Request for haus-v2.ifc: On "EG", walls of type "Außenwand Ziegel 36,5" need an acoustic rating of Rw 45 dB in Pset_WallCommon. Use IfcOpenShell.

First a look at what the model holds.

```python
import ifcopenshell
import ifcopenshell.util.element

model = ifcopenshell.open("haus-v2.ifc")
print(model.schema)
storey = next(s for s in model.by_type("IfcBuildingStorey") if s.Name == "EG")
walls = [e for e in ifcopenshell.util.element.get_decomposition(storey) if e.is_a("IfcWall")]
seen = {}
for e in walls:
    element_type = ifcopenshell.util.element.get_type(e)
    key = (element_type.Name if element_type != e and element_type else None, ifcopenshell.util.element.get_pset(e, "Pset_WallCommon", "AcousticRating"))
    seen[key] = seen.get(key, 0) + 1
for (name, value), count in sorted(seen.items(), key=str):
    print(count, "x", name, "|", value)
```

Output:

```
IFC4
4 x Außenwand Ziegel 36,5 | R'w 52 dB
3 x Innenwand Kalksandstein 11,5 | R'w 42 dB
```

```python
import ifcopenshell
import ifcopenshell.api.pset
import ifcopenshell.util.element

model = ifcopenshell.open("haus-v2.ifc")

storey = next(s for s in model.by_type("IfcBuildingStorey") if s.Name == "EG")
walls = [e for e in ifcopenshell.util.element.get_decomposition(storey) if e.is_a("IfcWall")]

count = 0
for e in walls:
    element_type = ifcopenshell.util.element.get_type(e)
    if element_type in (None, e) or element_type.Name != "Außenwand Ziegel 36,5":
        continue
    # add_pset returns the element's existing set when there is one.
    pset = ifcopenshell.api.pset.add_pset(model, product=e, name="Pset_WallCommon")
    ifcopenshell.api.pset.edit_pset(model, pset=pset, properties={"AcousticRating": "Rw 45 dB"})
    count += 1

print(count, "walls updated")

model.write("haus-v2_v2.ifc")
```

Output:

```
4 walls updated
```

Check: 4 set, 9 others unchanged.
